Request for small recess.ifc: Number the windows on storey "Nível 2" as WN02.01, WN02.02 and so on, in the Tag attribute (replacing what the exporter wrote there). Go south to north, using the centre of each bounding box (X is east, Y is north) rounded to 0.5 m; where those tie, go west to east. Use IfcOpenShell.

First a look at what the model holds.

```python
import ifcopenshell
import ifcopenshell.util.element
import ifcopenshell.util.placement

model = ifcopenshell.open("small recess.ifc")
print(model.schema)
storey = next(s for s in model.by_type("IfcBuildingStorey") if s.Name == "Nível 2")
windows = [e for e in ifcopenshell.util.element.get_decomposition(storey) if e.is_a("IfcWindow")]
for e in sorted(windows, key=lambda e: e.id()):
    origin = ifcopenshell.util.placement.get_local_placement(e.ObjectPlacement)[:3, 3]
    print(e.id(), e.Tag, e.Name, origin.round(2) + 0.0, sep=" | ")
```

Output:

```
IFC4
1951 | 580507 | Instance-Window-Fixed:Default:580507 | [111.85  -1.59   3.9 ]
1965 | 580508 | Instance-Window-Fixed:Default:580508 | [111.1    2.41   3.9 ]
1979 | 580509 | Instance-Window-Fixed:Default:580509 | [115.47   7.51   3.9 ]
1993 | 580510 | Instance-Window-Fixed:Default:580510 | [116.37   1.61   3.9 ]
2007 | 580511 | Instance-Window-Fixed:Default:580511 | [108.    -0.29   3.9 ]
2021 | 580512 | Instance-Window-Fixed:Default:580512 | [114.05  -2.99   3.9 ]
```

```python
import ifcopenshell
import ifcopenshell.geom
import ifcopenshell.util.element
import ifcopenshell.util.shape

model = ifcopenshell.open("small recess.ifc")
settings = ifcopenshell.geom.settings()
settings.set("use-world-coords", True)


def centre(element):
    shape = ifcopenshell.geom.create_shape(settings, element)
    return ifcopenshell.util.shape.get_bbox_centroid(shape.geometry)


storey = next(s for s in model.by_type("IfcBuildingStorey") if s.Name == "Nível 2")
windows = [e for e in ifcopenshell.util.element.get_decomposition(storey) if e.is_a("IfcWindow")]

# Insertion points can sit at a corner or the storey origin, so sort by the geometry (in metres).
centres = {e: centre(e) for e in windows}
windows.sort(key=lambda e: (round(centres[e][1] / 0.5), centres[e][0]))

for i, e in enumerate(windows, start=1):
    number = f"WN02.{i:02d}"
    e.Tag = number
    print(e.id(), number)

model.write("small recess_rev.ifc")
```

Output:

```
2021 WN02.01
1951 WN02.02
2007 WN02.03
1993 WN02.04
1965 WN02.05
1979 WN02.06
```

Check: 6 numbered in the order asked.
